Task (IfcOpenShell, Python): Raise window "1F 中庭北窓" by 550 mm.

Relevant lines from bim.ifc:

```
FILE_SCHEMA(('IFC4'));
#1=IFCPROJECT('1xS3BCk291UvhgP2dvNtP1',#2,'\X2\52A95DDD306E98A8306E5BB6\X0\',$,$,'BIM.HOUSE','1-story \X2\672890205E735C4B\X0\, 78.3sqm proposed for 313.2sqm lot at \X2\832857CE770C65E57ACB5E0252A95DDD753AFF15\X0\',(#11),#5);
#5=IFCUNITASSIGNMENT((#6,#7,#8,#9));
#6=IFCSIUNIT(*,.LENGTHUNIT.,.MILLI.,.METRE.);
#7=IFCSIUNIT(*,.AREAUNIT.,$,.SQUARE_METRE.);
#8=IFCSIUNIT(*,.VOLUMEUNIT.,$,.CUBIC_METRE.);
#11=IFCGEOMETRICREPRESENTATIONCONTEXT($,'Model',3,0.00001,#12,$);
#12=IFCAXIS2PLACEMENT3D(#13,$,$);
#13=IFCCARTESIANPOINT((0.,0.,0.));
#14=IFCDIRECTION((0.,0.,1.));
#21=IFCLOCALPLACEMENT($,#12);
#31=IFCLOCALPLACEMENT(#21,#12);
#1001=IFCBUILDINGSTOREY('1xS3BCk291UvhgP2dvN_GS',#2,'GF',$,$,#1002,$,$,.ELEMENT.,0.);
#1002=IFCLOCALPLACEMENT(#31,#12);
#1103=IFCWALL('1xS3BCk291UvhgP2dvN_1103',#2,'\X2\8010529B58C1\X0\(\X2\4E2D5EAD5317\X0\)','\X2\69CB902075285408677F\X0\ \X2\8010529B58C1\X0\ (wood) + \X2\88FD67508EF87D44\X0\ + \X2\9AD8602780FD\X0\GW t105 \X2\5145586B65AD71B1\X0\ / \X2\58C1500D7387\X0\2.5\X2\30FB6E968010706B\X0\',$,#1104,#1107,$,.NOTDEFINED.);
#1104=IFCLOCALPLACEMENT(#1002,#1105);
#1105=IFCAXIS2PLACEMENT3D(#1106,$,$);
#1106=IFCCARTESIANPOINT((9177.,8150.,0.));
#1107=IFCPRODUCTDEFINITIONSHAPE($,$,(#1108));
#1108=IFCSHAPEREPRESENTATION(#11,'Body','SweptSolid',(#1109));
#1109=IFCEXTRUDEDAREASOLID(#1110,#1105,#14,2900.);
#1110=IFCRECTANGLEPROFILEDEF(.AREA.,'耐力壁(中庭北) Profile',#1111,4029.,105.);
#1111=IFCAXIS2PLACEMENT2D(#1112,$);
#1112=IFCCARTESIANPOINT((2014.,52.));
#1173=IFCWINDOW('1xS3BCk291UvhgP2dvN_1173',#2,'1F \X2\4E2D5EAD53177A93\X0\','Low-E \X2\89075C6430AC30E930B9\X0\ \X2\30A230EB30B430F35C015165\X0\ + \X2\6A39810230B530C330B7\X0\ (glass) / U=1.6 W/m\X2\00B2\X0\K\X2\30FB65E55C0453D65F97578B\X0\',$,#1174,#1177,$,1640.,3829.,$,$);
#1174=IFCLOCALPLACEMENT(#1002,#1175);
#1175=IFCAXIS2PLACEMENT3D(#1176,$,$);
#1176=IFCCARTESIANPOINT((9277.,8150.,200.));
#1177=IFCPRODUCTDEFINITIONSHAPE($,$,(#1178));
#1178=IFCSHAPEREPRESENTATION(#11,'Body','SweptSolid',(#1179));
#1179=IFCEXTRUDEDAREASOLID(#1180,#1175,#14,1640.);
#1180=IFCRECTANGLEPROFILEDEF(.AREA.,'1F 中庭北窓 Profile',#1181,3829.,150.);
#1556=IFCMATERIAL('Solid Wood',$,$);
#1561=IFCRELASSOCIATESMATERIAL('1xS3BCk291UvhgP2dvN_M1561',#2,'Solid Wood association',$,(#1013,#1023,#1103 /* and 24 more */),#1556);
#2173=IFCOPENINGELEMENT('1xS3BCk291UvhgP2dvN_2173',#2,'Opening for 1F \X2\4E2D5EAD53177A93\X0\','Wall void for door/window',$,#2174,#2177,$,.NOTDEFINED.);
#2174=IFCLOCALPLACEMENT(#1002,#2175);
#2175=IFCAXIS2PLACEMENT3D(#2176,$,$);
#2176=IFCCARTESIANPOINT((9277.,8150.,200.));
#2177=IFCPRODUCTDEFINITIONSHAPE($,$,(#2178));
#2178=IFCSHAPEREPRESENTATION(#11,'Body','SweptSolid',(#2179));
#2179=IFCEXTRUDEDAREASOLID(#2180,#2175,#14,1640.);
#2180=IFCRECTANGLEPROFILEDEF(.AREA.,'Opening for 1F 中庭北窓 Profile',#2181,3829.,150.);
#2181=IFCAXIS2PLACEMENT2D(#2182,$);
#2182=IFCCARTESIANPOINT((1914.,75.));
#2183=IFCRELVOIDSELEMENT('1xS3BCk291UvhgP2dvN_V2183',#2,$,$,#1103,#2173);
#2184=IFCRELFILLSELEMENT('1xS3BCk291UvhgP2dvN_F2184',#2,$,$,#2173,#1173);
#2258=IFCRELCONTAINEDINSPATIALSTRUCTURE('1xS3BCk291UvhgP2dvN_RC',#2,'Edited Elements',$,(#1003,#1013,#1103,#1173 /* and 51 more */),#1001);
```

```python
import numpy as np
import ifcopenshell
import ifcopenshell.api.geometry
import ifcopenshell.util.placement
import ifcopenshell.util.unit

model = ifcopenshell.open("bim.ifc")
unit_scale = ifcopenshell.util.unit.calculate_unit_scale(model)

window = model.by_id(1173)
opening = window.FillsVoids[0].RelatingOpeningElement
dz = 0.55 / unit_scale

shift = np.array([0.0, 0.0, dz])
# The window is not placed relative to its opening, so move both.
for product in (opening, window):
    matrix = ifcopenshell.util.placement.get_local_placement(product.ObjectPlacement)
    matrix[:3, 3] += shift
    ifcopenshell.api.geometry.edit_object_placement(model, product=product, matrix=matrix, is_si=False)

print(f"moved by {dz * unit_scale:+.3f} m")

model.write("bim_edited.ifc")
```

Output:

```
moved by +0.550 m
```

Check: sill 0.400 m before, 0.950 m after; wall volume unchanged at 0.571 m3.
